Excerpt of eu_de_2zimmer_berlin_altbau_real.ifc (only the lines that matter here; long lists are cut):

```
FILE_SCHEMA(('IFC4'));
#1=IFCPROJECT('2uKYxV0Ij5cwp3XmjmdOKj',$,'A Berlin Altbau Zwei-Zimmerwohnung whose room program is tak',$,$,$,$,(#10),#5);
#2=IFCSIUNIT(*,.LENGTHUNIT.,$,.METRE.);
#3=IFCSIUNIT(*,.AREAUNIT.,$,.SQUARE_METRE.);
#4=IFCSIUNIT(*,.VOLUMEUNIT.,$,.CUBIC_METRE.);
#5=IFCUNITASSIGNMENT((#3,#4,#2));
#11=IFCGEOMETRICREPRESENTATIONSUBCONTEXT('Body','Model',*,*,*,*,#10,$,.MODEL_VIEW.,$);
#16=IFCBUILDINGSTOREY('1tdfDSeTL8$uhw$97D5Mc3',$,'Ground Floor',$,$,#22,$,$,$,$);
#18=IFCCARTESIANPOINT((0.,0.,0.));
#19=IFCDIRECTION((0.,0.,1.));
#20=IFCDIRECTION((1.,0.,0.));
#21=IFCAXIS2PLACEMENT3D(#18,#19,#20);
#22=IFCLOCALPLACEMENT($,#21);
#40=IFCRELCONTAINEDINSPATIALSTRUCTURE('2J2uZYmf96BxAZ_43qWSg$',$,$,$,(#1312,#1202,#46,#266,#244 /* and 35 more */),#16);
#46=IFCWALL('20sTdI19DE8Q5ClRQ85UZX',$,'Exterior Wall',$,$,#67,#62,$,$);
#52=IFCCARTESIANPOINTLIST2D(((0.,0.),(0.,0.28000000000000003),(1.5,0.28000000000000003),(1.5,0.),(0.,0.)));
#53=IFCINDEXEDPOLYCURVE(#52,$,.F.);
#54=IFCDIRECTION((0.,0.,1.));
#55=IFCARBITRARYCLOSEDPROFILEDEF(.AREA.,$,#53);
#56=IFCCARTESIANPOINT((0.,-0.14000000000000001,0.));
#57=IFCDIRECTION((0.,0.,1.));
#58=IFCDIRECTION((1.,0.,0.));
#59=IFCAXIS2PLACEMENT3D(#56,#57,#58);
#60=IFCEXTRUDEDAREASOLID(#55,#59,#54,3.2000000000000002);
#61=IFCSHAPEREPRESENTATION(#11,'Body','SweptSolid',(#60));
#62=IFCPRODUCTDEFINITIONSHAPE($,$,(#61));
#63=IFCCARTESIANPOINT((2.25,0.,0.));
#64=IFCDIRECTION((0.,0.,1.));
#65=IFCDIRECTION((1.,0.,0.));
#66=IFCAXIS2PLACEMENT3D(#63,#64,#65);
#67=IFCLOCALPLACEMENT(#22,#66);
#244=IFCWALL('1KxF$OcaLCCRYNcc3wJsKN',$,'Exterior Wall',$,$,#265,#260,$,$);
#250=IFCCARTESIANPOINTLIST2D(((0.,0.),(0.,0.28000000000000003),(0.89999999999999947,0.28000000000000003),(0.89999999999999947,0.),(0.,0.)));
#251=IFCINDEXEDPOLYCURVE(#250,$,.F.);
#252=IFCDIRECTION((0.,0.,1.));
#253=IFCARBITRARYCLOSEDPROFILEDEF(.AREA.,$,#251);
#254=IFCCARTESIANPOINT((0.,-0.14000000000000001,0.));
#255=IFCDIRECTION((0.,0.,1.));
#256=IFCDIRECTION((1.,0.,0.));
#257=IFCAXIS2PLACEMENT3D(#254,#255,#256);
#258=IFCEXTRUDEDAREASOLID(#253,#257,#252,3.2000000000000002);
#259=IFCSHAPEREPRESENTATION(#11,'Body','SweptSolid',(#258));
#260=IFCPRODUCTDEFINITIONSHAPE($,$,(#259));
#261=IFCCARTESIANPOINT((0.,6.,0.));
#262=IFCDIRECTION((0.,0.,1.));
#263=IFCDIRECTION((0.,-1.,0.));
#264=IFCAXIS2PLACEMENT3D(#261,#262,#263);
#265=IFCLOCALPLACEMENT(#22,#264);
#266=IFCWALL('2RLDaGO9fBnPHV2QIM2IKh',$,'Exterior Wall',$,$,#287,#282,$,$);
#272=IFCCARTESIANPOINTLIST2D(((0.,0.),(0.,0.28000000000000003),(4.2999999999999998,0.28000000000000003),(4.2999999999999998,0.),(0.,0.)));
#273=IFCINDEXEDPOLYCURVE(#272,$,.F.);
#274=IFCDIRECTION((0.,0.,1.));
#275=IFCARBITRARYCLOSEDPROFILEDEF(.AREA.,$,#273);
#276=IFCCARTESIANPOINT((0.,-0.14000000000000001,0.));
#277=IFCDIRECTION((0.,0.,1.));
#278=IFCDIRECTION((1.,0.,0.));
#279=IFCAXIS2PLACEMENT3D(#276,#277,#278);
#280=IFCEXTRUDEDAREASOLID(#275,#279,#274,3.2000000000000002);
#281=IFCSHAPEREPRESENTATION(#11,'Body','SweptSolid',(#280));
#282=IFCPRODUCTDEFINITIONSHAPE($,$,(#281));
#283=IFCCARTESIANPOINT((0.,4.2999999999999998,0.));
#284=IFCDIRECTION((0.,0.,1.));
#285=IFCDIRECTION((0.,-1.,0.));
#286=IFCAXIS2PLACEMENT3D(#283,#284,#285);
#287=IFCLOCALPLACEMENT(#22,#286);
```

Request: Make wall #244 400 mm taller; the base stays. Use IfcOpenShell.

```python
import ifcopenshell
import ifcopenshell.geom
import ifcopenshell.util.representation
import ifcopenshell.util.shape
import ifcopenshell.util.unit

model = ifcopenshell.open("eu_de_2zimmer_berlin_altbau_real.ifc")
unit_scale = ifcopenshell.util.unit.calculate_unit_scale(model)
settings = ifcopenshell.geom.settings()


def volume(element):
    """Net volume in cubic metres, openings subtracted."""
    shape = ifcopenshell.geom.create_shape(settings, element)
    return ifcopenshell.util.shape.get_volume(shape.geometry)


wall = model.by_guid("1KxF$OcaLCCRYNcc3wJsKN")
before = volume(wall)

body = ifcopenshell.util.representation.get_representation(wall, "Model", "Body")
solid = body.Items[0]
old_height = solid.Depth
solid.Depth += 0.4 / unit_scale
after = volume(wall)

print(f"height {old_height:g} -> {solid.Depth:g}, volume {before:.3f} -> {after:.3f} m3")

model.write("eu_de_2zimmer_berlin_altbau_real_v2.ifc")
```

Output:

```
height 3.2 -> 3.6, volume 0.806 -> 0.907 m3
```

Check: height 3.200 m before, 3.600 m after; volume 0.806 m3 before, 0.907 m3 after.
